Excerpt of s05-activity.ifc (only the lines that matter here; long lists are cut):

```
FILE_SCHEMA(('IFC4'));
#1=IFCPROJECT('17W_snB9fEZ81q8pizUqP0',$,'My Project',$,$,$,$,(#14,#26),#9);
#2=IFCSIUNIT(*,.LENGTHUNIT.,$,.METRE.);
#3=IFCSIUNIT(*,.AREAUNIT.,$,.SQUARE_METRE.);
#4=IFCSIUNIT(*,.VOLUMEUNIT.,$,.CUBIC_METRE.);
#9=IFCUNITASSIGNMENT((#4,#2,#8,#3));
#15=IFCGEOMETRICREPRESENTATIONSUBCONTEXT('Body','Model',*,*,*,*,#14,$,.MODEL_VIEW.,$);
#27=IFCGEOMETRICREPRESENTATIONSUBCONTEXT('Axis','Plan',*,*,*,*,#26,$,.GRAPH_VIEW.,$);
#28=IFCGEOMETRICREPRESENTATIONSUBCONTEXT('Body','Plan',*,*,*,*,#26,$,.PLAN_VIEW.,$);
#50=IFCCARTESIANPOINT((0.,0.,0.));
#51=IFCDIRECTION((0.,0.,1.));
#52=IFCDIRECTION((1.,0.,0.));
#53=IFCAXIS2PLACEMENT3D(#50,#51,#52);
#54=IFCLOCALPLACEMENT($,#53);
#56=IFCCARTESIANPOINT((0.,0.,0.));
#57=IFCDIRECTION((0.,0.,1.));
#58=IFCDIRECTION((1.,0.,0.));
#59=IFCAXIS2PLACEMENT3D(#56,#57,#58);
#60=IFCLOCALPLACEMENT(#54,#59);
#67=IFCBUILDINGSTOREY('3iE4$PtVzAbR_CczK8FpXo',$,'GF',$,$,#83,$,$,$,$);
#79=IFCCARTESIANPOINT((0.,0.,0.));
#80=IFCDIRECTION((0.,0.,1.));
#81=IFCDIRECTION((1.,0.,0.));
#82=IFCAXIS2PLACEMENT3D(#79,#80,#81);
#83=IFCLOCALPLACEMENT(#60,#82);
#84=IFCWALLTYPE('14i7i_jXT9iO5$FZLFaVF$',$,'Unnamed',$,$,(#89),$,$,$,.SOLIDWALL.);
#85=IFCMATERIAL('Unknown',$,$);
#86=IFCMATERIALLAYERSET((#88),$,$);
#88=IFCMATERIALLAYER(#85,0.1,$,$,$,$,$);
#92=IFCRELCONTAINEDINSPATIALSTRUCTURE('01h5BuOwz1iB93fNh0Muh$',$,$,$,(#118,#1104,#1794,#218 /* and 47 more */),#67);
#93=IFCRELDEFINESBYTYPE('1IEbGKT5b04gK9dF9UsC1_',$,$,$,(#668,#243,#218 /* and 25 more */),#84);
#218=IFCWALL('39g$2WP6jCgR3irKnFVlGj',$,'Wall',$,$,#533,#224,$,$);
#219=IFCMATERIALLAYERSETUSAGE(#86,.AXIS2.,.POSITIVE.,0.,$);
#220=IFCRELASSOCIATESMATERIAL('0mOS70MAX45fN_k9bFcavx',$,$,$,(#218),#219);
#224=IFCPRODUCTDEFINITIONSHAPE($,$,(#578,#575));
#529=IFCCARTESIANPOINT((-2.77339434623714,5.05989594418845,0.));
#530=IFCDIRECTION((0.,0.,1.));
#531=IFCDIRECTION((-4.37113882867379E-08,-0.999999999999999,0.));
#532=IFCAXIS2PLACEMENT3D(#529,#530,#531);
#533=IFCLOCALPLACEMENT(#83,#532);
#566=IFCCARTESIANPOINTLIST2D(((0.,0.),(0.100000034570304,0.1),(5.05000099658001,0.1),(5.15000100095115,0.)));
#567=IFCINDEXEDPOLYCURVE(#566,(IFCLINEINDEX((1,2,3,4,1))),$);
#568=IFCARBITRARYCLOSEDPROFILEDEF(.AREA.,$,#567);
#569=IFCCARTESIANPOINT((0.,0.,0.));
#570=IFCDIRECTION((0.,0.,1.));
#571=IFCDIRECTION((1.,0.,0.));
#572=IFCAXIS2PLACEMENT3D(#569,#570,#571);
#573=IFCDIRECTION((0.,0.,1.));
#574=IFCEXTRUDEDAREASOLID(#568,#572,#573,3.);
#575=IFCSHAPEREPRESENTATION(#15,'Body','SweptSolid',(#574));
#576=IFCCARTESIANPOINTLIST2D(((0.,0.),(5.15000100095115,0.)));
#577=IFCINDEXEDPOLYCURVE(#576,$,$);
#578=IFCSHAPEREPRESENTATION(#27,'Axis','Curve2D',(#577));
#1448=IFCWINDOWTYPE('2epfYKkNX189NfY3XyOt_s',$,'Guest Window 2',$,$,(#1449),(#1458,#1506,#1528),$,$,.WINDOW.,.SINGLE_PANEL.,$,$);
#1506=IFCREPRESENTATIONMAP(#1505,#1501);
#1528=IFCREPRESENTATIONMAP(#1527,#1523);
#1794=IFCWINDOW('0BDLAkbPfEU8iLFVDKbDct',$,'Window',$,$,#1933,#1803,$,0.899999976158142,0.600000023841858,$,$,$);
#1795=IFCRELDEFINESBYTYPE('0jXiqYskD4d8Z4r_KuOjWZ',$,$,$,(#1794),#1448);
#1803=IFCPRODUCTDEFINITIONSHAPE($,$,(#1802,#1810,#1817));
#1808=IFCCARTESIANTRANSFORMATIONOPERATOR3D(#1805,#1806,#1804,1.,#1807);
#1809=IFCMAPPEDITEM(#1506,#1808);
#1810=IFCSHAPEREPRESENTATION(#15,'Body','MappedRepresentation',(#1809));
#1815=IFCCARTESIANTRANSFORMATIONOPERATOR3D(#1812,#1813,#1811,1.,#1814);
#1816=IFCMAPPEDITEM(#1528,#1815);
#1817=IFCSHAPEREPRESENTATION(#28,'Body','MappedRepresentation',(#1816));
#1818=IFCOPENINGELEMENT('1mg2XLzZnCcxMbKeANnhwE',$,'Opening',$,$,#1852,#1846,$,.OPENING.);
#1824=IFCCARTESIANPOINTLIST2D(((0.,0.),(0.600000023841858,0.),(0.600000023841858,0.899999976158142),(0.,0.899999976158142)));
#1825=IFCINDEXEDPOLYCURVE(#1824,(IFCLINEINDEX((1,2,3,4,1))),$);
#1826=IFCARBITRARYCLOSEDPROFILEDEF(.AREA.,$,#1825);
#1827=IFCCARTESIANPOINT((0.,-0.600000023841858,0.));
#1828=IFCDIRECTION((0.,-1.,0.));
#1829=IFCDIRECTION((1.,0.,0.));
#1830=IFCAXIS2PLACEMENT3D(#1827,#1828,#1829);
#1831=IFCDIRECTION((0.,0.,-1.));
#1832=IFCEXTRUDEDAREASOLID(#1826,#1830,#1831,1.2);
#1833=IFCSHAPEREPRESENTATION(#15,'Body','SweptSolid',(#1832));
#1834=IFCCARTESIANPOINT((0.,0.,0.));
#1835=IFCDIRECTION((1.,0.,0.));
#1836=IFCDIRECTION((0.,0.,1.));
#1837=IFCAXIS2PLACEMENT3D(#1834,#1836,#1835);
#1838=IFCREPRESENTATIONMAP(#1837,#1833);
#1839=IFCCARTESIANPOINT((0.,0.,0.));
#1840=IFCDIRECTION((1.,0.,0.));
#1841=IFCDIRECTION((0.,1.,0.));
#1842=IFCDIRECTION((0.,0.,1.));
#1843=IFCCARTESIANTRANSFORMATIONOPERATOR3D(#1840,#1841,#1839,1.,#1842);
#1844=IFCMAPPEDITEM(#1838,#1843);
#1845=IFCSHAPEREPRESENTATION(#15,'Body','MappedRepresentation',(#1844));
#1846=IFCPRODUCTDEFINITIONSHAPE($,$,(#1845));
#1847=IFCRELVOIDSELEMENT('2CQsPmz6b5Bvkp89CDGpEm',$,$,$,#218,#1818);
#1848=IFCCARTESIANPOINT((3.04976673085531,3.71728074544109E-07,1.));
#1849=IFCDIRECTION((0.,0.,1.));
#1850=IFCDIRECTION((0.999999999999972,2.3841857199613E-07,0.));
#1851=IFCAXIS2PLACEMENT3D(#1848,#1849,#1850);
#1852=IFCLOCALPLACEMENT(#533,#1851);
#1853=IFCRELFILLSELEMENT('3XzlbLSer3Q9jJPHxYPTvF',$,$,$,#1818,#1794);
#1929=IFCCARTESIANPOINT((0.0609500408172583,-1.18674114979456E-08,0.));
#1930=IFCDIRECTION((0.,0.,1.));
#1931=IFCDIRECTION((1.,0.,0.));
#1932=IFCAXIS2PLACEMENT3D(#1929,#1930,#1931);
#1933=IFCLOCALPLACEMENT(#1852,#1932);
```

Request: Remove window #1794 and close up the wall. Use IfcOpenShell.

```python
import ifcopenshell
import ifcopenshell.api.feature
import ifcopenshell.api.root
import ifcopenshell.geom
import ifcopenshell.util.shape

model = ifcopenshell.open("s05-activity.ifc")
settings = ifcopenshell.geom.settings()


def volume(element):
    """Net volume in cubic metres, openings subtracted."""
    shape = ifcopenshell.geom.create_shape(settings, element)
    return ifcopenshell.util.shape.get_volume(shape.geometry)


window = model.by_guid("0BDLAkbPfEU8iLFVDKbDct")
opening = window.FillsVoids[0].RelatingOpeningElement
wall = opening.VoidsElements[0].RelatingBuildingElement
before = volume(wall)

ifcopenshell.api.root.remove_product(model, product=window)
ifcopenshell.api.feature.remove_feature(model, feature=opening)

after = volume(wall)

print(f"wall volume {before:.3f} -> {after:.3f} m3")

model.write("s05-activity_rev.ifc")
```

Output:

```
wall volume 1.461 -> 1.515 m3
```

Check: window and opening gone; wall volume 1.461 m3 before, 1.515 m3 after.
